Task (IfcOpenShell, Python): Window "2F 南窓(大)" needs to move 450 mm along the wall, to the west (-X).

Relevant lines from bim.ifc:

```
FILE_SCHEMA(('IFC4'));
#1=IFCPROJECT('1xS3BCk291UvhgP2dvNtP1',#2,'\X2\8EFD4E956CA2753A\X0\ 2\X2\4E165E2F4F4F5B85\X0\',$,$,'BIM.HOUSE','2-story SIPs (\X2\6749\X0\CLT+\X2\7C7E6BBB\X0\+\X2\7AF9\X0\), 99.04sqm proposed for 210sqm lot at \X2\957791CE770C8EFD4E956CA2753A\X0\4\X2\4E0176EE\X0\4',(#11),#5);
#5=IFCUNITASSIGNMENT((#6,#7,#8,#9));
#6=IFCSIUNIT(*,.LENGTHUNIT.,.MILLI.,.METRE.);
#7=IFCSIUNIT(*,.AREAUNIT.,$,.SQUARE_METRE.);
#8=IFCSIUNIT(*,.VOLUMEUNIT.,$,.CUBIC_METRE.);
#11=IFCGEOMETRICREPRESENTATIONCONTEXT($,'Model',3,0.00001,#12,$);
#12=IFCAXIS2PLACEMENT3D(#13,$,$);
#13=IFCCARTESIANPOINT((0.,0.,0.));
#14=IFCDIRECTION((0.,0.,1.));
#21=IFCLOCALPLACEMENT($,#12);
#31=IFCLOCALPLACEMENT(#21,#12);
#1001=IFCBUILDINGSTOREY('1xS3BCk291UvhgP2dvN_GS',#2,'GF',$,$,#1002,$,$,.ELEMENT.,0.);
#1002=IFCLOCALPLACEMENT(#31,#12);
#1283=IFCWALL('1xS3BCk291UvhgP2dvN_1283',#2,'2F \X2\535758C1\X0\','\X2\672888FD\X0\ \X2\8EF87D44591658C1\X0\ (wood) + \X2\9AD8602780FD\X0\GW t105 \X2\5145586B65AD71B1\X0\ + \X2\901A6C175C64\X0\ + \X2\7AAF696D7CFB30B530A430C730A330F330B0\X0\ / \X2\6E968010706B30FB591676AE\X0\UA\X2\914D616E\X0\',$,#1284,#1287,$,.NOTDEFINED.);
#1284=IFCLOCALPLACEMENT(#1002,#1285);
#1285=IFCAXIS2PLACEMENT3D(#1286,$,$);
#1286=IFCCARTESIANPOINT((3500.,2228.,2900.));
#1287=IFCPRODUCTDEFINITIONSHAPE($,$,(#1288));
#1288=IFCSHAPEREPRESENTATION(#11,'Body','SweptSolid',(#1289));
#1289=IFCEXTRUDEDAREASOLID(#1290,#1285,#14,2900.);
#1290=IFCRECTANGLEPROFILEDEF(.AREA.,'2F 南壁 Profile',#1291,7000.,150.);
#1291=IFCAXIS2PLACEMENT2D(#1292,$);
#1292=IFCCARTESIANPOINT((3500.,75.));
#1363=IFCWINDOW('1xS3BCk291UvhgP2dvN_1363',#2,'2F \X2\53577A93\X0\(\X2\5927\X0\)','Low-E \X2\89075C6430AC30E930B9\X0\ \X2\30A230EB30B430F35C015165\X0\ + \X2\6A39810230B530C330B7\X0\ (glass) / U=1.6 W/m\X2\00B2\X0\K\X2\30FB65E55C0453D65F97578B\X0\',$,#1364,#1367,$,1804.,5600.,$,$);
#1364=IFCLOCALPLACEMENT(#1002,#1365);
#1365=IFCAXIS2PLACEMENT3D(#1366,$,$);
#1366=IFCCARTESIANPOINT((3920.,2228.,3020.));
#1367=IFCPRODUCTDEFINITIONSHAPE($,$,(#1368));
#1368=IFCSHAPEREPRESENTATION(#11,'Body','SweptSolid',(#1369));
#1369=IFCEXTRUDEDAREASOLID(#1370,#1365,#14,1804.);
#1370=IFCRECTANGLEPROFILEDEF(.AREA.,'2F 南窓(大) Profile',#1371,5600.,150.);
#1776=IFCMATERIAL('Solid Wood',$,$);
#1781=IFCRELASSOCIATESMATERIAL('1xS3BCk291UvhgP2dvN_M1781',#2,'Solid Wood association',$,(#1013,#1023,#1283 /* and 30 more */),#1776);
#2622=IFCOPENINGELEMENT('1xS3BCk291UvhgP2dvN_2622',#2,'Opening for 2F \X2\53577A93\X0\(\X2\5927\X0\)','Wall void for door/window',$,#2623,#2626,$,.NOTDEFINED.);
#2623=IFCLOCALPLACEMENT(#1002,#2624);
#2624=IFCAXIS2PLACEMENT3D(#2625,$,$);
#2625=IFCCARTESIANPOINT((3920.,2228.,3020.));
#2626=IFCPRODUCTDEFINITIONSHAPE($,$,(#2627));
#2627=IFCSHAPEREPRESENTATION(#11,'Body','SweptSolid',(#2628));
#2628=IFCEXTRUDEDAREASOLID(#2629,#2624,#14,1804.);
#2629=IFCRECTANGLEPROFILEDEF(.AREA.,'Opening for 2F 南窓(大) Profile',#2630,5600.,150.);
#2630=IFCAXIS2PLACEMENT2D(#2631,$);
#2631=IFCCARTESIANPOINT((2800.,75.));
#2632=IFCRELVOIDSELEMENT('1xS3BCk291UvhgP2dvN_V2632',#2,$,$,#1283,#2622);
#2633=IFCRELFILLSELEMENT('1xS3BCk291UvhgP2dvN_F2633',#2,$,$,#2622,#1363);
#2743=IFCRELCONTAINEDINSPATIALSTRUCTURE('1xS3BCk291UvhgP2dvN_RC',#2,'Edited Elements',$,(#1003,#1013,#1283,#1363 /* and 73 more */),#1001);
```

```python
import ifcopenshell
import ifcopenshell.api.geometry
import ifcopenshell.util.placement

model = ifcopenshell.open("bim.ifc")

window = model.by_guid("1xS3BCk291UvhgP2dvN_1363")
opening = window.FillsVoids[0].RelatingOpeningElement
wall = opening.VoidsElements[0].RelatingBuildingElement

wall_matrix = ifcopenshell.util.placement.get_local_placement(wall.ObjectPlacement)
shift = wall_matrix[:3, 0] * -450.0
before = ifcopenshell.util.placement.get_local_placement(window.ObjectPlacement)[:3, 3].copy()

# The window is not placed relative to its opening, so move both.
for product in (opening, window):
    matrix = ifcopenshell.util.placement.get_local_placement(product.ObjectPlacement)
    matrix[:3, 3] += shift
    ifcopenshell.api.geometry.edit_object_placement(model, product=product, matrix=matrix, is_si=False)

after = ifcopenshell.util.placement.get_local_placement(window.ObjectPlacement)[:3, 3]
print("window moved by", (after - before).round(3) + 0.0)

model.write("bim_edited.ifc")
```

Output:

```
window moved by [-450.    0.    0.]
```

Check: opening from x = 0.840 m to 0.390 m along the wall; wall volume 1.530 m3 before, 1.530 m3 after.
